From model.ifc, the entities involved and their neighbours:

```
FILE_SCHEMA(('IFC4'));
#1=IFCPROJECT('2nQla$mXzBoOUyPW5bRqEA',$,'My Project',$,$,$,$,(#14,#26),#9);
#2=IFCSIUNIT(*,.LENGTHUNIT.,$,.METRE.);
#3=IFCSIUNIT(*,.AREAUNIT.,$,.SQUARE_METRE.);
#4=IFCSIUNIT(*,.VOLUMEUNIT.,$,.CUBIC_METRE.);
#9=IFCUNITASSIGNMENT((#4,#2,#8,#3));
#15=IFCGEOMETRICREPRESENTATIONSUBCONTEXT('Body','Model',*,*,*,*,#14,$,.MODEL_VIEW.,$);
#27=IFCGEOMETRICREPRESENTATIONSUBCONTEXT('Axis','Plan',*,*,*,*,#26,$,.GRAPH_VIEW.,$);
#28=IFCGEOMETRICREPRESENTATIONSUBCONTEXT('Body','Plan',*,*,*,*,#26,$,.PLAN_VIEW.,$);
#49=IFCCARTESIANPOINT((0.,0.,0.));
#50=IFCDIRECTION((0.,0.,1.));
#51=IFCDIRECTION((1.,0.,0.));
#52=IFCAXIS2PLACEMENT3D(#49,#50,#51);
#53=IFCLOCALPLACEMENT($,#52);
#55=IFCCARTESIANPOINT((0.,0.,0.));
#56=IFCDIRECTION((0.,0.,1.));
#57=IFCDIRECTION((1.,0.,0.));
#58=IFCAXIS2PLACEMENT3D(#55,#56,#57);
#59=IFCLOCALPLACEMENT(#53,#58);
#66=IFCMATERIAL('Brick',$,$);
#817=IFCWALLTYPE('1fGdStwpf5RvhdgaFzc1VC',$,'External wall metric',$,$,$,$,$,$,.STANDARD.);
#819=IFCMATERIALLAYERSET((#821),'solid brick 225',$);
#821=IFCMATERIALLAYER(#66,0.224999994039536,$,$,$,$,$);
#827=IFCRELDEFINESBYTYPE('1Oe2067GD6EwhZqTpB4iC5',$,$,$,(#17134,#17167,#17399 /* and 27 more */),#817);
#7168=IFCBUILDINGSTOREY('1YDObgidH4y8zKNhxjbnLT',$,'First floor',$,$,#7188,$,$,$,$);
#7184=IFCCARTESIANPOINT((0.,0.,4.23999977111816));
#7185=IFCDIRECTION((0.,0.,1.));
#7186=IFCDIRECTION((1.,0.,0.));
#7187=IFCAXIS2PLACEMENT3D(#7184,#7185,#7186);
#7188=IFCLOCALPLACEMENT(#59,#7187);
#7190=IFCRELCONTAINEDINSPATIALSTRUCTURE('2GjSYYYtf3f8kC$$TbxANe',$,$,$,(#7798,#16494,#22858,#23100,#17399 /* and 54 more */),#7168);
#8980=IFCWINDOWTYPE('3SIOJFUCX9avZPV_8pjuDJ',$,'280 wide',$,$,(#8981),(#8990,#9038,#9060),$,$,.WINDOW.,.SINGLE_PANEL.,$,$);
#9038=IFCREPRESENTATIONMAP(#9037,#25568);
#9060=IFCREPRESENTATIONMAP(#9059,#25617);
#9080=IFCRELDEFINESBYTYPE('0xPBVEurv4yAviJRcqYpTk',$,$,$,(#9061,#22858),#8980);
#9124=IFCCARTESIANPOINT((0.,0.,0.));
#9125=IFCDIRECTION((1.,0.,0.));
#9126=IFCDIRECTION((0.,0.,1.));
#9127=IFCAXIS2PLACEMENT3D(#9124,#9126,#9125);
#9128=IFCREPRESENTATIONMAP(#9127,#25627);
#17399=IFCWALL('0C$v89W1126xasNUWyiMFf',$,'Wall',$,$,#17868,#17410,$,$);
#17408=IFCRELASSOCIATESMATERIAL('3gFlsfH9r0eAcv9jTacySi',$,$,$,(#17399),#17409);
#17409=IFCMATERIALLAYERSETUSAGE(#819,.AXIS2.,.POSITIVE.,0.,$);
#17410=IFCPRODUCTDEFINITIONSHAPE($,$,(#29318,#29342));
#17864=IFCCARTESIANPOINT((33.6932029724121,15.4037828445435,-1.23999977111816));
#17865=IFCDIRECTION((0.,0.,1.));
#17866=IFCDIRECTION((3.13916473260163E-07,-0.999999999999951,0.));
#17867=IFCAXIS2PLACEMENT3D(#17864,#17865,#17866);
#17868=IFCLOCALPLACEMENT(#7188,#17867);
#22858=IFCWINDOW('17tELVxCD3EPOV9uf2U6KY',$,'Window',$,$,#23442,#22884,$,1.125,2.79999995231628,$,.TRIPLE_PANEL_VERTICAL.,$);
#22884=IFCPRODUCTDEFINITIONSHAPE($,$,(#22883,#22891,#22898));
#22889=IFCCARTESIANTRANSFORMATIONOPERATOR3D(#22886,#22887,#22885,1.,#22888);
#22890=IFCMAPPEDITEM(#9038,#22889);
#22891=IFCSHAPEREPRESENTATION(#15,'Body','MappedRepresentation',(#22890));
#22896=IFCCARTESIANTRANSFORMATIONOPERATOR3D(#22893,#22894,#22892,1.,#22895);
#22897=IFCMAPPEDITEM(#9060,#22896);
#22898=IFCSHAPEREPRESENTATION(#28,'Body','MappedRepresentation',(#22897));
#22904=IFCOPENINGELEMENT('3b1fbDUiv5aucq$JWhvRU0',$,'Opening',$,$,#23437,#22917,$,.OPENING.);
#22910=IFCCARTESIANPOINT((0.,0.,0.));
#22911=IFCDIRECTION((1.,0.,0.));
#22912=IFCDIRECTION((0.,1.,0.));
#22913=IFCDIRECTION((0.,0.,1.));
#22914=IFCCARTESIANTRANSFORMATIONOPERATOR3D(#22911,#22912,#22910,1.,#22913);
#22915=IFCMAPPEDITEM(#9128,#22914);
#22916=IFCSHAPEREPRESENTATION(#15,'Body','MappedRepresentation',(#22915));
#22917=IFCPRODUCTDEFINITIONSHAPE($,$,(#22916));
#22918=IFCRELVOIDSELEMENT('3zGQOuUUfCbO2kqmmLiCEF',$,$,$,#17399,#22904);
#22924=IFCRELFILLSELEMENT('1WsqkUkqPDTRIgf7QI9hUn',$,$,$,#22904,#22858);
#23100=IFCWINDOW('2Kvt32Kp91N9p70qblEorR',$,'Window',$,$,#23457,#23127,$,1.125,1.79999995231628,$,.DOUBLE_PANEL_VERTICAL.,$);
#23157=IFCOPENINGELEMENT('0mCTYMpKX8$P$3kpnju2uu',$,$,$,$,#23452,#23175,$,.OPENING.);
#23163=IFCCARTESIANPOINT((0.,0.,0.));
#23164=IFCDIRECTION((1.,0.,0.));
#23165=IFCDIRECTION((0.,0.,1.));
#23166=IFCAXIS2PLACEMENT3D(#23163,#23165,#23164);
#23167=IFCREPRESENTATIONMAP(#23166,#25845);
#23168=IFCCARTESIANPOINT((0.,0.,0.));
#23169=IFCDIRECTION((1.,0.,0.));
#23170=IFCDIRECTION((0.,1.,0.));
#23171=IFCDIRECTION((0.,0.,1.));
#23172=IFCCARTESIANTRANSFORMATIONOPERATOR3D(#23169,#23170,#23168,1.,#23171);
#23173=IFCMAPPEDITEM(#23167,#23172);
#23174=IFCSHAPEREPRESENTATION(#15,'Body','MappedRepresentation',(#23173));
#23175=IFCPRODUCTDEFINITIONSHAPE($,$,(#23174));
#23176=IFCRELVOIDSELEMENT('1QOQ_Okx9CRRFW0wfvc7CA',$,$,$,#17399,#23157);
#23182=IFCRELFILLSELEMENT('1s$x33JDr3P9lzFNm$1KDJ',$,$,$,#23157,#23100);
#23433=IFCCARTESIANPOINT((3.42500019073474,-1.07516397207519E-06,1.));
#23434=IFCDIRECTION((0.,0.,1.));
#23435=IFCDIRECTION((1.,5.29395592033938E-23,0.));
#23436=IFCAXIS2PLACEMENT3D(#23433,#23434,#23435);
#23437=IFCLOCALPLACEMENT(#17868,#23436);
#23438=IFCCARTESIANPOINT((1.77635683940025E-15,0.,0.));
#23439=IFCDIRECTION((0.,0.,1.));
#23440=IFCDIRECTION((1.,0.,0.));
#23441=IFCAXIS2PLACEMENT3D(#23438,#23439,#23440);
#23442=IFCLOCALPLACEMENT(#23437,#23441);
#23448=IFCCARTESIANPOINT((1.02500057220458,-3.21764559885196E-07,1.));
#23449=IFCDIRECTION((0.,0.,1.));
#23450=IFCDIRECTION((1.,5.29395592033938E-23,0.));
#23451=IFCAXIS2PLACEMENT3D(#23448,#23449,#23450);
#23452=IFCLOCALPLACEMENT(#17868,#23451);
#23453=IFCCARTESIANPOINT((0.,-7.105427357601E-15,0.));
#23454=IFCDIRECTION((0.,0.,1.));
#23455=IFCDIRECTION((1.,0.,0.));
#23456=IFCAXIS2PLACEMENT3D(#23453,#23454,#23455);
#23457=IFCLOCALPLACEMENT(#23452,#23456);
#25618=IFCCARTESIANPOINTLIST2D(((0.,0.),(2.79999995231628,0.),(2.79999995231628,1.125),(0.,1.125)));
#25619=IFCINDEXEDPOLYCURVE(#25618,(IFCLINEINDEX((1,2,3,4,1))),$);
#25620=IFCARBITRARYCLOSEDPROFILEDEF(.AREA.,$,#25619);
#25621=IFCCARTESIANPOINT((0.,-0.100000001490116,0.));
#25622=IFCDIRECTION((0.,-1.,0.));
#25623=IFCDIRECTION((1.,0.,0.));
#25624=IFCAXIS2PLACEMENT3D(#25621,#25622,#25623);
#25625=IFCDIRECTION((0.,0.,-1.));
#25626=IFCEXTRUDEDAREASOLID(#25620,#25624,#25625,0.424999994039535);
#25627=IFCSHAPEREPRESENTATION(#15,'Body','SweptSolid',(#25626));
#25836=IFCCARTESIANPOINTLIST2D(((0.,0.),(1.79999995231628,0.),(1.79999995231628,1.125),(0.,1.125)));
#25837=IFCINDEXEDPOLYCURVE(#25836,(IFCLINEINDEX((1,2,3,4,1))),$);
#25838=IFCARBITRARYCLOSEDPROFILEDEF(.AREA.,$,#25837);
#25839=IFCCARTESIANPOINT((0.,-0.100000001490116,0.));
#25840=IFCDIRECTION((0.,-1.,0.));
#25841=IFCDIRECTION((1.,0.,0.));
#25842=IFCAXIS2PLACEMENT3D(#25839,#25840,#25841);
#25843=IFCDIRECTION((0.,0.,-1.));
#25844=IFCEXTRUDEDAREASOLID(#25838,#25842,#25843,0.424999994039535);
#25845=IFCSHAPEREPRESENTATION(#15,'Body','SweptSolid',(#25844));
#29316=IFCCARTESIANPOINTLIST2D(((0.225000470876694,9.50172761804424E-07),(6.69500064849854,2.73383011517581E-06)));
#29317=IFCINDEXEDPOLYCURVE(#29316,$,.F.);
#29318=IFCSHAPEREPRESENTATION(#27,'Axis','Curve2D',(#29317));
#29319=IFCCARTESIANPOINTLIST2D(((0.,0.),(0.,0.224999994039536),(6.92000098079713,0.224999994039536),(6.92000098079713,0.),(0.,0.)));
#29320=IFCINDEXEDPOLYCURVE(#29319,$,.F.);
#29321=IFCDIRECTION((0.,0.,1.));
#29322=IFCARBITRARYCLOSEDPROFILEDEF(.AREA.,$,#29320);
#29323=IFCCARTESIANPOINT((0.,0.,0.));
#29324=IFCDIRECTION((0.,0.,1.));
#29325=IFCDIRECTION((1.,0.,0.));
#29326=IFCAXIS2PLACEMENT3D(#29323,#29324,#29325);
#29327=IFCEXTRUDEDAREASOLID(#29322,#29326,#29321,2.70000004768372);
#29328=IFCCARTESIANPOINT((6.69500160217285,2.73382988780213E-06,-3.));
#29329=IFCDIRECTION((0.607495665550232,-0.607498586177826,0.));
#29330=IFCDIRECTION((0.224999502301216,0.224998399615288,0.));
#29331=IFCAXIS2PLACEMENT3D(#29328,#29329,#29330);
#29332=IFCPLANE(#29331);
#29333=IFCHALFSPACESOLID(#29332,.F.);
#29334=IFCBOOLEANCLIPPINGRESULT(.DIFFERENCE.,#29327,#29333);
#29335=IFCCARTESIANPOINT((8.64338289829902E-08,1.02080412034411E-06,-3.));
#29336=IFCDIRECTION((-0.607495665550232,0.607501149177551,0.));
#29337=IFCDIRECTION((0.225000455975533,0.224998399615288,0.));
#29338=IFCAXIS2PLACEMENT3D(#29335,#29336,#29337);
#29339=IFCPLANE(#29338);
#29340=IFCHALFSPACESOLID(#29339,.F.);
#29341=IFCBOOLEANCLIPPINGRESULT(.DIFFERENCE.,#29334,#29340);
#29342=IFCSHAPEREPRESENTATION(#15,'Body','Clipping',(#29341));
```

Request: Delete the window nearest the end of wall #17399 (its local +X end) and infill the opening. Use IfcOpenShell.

```python
import ifcopenshell
import ifcopenshell.api.feature
import ifcopenshell.api.root
import ifcopenshell.geom
import ifcopenshell.util.shape

model = ifcopenshell.open("model.ifc")
settings = ifcopenshell.geom.settings()


def volume(element):
    """Net volume in cubic metres, openings subtracted."""
    shape = ifcopenshell.geom.create_shape(settings, element)
    return ifcopenshell.util.shape.get_volume(shape.geometry)


window = model.by_id(22858)
opening = window.FillsVoids[0].RelatingOpeningElement
wall = opening.VoidsElements[0].RelatingBuildingElement
before = volume(wall)

ifcopenshell.api.root.remove_product(model, product=window)
ifcopenshell.api.feature.remove_feature(model, feature=opening)

after = volume(wall)

print(f"wall volume {before:.3f} -> {after:.3f} m3")

model.write("model-out.ifc")
```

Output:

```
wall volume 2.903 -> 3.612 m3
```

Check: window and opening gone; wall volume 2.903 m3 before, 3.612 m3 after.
